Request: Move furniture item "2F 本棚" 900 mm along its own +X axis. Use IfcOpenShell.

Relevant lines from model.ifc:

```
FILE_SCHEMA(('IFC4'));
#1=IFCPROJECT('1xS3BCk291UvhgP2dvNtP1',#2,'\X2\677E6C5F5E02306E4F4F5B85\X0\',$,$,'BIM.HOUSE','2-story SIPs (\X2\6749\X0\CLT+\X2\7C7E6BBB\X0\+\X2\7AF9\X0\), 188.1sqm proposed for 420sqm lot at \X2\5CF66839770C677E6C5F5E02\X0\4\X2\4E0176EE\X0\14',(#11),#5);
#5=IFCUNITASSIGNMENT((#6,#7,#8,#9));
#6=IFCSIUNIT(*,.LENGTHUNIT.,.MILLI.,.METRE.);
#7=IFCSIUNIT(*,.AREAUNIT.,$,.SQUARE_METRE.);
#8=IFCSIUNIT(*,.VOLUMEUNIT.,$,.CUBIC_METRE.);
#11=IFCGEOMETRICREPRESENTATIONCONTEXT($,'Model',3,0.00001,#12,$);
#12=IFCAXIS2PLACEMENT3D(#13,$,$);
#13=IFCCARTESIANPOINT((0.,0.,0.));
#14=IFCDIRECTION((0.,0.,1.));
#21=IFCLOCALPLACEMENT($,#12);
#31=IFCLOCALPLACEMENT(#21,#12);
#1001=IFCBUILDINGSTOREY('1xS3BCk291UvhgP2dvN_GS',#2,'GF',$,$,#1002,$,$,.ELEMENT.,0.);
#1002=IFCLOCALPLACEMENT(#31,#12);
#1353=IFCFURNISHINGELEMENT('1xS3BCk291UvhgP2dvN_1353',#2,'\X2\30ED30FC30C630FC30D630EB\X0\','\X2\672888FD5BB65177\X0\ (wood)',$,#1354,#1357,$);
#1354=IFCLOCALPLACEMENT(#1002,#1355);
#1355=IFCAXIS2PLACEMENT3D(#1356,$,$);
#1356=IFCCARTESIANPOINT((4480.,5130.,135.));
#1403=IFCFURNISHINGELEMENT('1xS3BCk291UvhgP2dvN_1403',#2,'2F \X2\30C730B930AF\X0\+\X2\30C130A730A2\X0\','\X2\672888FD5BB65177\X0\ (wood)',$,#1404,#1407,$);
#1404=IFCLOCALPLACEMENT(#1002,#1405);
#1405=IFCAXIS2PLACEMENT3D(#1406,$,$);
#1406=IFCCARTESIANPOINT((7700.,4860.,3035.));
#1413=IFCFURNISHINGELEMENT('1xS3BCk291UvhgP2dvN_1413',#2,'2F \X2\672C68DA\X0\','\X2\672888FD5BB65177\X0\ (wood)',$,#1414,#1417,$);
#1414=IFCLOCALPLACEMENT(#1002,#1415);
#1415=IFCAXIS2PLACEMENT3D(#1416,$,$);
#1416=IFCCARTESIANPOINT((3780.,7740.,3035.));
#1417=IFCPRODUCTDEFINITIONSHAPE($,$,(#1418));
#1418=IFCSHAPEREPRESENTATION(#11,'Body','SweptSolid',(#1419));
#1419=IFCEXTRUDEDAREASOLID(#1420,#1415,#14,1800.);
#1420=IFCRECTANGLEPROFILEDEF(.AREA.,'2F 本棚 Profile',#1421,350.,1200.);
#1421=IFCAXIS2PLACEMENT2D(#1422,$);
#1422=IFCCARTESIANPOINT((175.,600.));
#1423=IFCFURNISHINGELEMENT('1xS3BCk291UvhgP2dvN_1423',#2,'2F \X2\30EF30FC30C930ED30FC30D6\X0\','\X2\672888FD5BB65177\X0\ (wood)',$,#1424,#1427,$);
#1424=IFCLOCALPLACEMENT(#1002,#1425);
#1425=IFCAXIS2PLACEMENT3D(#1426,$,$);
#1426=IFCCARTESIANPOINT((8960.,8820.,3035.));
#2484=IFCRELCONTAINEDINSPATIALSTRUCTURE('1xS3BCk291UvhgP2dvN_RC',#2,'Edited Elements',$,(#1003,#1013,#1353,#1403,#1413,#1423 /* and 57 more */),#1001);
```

```python
import ifcopenshell
import ifcopenshell.api.geometry
import ifcopenshell.util.placement
import ifcopenshell.util.unit

model = ifcopenshell.open("model.ifc")
unit_scale = ifcopenshell.util.unit.calculate_unit_scale(model)

item = model.by_id(1413)
matrix = ifcopenshell.util.placement.get_local_placement(item.ObjectPlacement)
matrix[:3, 3] += matrix[:3, 0] * 0.9 / unit_scale
ifcopenshell.api.geometry.edit_object_placement(model, product=item, matrix=matrix, is_si=False)

print(ifcopenshell.util.placement.get_local_placement(item.ObjectPlacement).round(3) + 0.0)

model.write("model_v2.ifc")
```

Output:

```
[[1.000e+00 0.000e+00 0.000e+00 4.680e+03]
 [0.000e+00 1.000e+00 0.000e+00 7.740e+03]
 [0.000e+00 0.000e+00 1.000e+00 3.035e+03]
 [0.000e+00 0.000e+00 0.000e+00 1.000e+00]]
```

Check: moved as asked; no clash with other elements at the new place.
